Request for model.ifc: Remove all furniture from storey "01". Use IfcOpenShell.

First a look at what the model holds.

```python
import ifcopenshell
import ifcopenshell.util.element

model = ifcopenshell.open("model.ifc")
print(model.schema)
storey = next(s for s in model.by_type("IfcBuildingStorey") if s.Name == "01")
furniture = [e for e in ifcopenshell.util.element.get_decomposition(storey) if e.is_a("IfcFurnishingElement")]
seen = {}
for e in furniture:
    element_type = ifcopenshell.util.element.get_type(e)
    name = element_type.Name if element_type not in (None, e) else None
    seen[name] = seen.get(name, 0) + 1
for name, count in sorted(seen.items(), key=str):
    print(count, "x", name)
```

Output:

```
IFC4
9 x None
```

```python
import ifcopenshell
import ifcopenshell.api.root
import ifcopenshell.util.element

model = ifcopenshell.open("model.ifc")

storey = next(s for s in model.by_type("IfcBuildingStorey") if s.Name == "01")
furniture = [e for e in ifcopenshell.util.element.get_decomposition(storey) if e.is_a("IfcFurnishingElement")]

for e in furniture:
    ifcopenshell.api.root.remove_product(model, product=e)
print(len(furniture), "removed")

model.write("model_v2.ifc")
```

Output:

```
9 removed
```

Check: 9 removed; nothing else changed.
